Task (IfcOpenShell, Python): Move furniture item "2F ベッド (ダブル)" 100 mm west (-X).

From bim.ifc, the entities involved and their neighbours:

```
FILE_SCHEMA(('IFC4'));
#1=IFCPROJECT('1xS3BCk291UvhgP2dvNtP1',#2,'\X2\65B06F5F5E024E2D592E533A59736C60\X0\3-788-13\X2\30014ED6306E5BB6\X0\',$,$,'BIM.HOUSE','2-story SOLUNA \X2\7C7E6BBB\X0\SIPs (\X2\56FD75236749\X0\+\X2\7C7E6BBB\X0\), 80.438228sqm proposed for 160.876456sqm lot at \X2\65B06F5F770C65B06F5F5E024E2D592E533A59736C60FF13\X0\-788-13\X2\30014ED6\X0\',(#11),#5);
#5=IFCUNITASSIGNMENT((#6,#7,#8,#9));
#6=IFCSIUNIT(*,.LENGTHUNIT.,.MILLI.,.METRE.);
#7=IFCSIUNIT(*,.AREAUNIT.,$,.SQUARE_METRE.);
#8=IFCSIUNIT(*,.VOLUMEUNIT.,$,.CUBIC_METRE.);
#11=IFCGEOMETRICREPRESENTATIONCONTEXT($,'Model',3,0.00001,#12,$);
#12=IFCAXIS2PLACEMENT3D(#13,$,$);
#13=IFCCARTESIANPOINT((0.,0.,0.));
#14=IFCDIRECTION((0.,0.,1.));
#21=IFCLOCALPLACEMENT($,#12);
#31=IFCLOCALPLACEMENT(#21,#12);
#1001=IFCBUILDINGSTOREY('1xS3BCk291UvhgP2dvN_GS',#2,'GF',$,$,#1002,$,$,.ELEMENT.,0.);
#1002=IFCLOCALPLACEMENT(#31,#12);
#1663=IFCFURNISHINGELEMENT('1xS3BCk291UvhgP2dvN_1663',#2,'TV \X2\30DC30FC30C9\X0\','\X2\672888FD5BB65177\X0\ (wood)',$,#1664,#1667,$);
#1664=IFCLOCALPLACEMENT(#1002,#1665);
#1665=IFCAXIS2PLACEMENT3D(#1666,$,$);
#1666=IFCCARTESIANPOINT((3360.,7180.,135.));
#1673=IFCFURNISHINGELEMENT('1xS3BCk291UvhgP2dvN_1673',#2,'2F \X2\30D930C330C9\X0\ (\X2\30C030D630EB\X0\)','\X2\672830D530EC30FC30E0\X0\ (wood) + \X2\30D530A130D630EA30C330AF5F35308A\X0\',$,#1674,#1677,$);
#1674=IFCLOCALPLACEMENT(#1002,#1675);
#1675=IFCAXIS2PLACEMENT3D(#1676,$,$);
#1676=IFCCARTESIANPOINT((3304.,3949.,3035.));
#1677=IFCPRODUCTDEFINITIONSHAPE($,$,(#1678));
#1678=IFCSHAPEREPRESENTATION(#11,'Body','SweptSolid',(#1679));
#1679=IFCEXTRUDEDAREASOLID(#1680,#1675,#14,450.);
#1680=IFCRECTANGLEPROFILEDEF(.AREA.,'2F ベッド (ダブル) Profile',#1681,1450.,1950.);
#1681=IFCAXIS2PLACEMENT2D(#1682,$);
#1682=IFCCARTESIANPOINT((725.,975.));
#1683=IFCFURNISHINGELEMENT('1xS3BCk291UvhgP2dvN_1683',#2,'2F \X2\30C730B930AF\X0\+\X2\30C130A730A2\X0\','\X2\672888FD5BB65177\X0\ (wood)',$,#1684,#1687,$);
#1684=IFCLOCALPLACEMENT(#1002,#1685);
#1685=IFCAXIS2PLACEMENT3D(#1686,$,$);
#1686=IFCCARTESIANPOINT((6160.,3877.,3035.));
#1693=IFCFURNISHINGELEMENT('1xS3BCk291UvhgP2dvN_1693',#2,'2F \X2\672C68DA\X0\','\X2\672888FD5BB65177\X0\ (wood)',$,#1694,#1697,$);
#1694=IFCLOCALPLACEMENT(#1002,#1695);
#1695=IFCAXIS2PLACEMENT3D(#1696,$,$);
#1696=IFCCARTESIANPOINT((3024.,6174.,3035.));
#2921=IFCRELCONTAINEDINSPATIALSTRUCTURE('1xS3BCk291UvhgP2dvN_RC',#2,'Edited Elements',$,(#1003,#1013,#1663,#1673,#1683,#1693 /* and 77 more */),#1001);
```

```python
import ifcopenshell
import ifcopenshell.api.geometry
import ifcopenshell.util.placement

model = ifcopenshell.open("bim.ifc")

item = model.by_guid("1xS3BCk291UvhgP2dvN_1673")
matrix = ifcopenshell.util.placement.get_local_placement(item.ObjectPlacement)
matrix[0, 3] -= 100.0
ifcopenshell.api.geometry.edit_object_placement(model, product=item, matrix=matrix, is_si=False)

print(ifcopenshell.util.placement.get_local_placement(item.ObjectPlacement).round(3) + 0.0)

model.write("bim_rev.ifc")
```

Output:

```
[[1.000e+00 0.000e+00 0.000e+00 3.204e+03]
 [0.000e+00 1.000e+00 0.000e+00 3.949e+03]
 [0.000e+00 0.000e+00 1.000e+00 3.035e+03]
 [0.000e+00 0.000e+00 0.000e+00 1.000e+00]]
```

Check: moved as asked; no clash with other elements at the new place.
